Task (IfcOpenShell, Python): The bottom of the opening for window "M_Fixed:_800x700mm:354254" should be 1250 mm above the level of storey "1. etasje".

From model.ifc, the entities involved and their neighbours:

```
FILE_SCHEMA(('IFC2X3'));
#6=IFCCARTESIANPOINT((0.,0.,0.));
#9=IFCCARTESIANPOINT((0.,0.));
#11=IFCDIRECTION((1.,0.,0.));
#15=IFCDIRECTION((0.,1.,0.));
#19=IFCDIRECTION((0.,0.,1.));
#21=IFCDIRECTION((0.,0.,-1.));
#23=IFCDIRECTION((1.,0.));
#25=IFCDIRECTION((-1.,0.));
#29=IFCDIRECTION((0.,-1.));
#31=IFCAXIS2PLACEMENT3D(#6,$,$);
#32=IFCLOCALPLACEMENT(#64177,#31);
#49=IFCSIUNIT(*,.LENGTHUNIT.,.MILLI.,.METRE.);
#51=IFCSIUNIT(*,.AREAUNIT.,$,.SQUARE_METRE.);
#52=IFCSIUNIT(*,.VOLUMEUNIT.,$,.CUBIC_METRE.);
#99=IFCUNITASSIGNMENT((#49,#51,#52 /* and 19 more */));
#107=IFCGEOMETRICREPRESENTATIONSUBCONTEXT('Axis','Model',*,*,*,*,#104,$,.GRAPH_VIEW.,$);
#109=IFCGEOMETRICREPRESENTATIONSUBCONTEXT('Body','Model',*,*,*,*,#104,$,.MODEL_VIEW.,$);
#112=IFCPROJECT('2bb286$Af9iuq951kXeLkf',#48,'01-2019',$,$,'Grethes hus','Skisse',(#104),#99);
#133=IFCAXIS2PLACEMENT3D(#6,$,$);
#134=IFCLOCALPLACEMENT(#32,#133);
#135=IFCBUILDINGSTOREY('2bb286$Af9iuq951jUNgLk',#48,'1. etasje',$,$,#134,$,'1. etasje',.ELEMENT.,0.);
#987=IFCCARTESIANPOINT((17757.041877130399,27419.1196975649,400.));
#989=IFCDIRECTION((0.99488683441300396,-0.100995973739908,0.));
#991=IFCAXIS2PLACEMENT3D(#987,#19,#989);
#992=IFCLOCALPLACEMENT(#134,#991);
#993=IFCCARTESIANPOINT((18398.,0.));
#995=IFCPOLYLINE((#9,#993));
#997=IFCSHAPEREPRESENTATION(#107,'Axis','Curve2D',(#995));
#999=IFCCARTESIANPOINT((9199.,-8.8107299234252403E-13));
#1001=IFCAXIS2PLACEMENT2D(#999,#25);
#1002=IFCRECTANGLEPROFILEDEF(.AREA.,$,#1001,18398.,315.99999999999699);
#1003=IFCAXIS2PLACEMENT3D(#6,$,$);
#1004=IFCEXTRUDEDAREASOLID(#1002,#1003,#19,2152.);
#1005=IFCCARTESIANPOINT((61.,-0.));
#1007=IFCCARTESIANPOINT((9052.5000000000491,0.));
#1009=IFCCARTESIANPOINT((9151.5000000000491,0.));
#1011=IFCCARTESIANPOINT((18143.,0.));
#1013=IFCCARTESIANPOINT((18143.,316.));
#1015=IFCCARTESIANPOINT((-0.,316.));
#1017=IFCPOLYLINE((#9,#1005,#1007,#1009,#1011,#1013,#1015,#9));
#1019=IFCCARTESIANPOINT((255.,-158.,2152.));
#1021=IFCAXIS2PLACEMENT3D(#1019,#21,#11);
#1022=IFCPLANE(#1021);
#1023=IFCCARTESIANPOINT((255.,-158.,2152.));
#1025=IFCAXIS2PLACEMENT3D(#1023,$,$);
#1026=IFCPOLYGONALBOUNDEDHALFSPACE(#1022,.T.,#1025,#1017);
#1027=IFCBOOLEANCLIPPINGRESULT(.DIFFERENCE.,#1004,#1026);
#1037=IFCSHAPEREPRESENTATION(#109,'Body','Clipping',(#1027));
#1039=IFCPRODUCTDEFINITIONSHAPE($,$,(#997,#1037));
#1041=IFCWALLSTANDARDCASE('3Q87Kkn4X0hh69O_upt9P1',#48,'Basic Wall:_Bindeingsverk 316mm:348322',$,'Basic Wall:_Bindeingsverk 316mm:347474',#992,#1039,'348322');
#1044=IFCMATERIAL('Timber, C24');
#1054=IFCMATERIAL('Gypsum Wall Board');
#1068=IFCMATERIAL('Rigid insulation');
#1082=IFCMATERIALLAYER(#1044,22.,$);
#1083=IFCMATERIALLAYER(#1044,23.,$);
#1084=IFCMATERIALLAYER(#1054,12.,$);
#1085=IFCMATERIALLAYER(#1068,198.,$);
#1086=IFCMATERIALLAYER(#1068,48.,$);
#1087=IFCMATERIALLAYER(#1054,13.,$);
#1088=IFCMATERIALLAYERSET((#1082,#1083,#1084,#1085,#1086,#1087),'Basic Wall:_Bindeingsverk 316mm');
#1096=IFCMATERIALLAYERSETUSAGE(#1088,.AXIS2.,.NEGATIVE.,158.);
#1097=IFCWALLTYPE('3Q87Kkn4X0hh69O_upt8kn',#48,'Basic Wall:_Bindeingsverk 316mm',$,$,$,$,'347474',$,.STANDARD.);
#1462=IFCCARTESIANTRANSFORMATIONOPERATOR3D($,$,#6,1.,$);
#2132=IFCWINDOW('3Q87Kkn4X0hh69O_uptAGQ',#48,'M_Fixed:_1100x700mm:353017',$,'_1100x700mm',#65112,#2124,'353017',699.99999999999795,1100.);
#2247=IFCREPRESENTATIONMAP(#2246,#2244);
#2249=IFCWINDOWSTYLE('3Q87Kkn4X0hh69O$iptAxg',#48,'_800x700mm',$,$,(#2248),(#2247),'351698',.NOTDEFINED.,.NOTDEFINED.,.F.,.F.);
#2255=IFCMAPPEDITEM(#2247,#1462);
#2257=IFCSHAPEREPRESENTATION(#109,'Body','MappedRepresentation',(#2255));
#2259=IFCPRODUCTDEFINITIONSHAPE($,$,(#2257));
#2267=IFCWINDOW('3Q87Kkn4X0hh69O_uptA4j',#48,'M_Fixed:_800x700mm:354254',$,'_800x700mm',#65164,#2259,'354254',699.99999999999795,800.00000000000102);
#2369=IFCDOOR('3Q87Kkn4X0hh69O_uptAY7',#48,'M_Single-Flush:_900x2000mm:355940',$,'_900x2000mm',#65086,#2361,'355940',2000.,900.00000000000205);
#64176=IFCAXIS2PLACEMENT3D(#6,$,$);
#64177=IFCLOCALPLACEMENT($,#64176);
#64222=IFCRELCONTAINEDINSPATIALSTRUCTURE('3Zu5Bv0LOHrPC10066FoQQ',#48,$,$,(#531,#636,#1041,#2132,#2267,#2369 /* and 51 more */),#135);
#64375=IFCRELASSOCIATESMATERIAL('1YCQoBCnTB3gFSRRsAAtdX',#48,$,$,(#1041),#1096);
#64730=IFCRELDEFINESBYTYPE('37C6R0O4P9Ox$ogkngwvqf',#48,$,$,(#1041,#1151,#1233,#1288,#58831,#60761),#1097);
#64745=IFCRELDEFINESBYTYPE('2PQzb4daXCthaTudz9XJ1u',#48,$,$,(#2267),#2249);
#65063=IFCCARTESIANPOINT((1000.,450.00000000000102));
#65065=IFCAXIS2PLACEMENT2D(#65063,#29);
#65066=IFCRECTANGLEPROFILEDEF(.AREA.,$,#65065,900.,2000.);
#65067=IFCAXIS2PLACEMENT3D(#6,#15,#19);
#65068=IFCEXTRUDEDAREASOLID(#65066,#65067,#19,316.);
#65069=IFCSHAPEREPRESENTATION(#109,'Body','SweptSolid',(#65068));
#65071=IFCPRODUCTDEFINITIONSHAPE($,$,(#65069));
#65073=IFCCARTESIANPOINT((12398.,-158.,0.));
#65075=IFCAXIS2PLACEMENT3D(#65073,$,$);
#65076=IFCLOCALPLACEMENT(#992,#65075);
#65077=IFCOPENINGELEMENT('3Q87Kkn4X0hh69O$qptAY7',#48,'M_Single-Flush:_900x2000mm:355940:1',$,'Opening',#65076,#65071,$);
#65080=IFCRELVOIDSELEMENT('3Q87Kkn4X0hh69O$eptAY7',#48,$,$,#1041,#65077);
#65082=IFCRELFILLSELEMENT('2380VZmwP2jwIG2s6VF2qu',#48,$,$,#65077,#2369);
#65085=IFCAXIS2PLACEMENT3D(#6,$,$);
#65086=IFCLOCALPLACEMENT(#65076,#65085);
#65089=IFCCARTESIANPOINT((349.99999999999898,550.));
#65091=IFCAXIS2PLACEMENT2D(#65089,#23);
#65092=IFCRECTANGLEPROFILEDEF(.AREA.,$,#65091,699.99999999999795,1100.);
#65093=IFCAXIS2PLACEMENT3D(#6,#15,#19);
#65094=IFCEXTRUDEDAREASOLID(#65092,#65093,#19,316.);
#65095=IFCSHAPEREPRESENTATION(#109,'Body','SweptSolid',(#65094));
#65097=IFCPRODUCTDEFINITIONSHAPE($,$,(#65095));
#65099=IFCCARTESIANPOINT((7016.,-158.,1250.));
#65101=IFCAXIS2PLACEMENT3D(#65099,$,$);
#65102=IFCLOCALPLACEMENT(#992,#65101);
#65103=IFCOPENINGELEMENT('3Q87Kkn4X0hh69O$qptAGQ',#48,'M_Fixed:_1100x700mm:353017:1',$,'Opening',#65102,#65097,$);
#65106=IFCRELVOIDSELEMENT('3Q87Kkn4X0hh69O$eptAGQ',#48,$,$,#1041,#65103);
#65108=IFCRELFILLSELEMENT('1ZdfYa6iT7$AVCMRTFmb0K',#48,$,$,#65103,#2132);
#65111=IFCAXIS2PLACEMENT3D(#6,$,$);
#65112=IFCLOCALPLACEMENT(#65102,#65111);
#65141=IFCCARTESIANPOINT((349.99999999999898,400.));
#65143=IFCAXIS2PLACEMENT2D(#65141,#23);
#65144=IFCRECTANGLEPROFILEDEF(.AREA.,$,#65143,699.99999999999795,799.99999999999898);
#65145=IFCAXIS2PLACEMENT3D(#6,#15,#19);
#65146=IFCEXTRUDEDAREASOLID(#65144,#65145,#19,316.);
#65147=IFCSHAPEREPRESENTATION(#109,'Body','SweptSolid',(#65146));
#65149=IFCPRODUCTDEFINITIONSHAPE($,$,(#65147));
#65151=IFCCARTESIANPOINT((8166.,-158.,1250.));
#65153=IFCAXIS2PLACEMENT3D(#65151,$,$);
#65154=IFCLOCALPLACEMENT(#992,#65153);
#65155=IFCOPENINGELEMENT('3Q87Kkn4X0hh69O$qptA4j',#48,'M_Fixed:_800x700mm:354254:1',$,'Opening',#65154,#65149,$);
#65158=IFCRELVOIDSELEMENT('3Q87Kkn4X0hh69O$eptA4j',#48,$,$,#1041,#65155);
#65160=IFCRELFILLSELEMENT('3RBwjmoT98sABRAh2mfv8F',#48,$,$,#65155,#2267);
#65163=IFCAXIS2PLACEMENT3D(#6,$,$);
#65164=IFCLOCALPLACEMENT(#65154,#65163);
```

```python
import numpy as np
import ifcopenshell
import ifcopenshell.api.geometry
import ifcopenshell.geom
import ifcopenshell.util.element
import ifcopenshell.util.placement
import ifcopenshell.util.shape
import ifcopenshell.util.unit

model = ifcopenshell.open("model.ifc")
unit_scale = ifcopenshell.util.unit.calculate_unit_scale(model)

window = model.by_id(2267)
opening = window.FillsVoids[0].RelatingOpeningElement
storey = ifcopenshell.util.element.get_container(window, ifc_class="IfcBuildingStorey")
level = ifcopenshell.util.placement.get_local_placement(storey.ObjectPlacement)[2, 3]

# The opening's origin need not be at the sill, so measure its lowest point.
shape = ifcopenshell.geom.create_shape(ifcopenshell.geom.settings(), opening)
bottom = ifcopenshell.util.shape.get_shape_bottom_elevation(shape, shape.geometry) / unit_scale
dz = level + 1250.0 - bottom

shift = np.array([0.0, 0.0, dz])
# The window is placed relative to its opening, so it follows when the opening moves.
matrix = ifcopenshell.util.placement.get_local_placement(opening.ObjectPlacement)
matrix[:3, 3] += shift
ifcopenshell.api.geometry.edit_object_placement(
    model, product=opening, matrix=matrix, is_si=False, should_transform_children=True
)

print(f"moved by {dz * unit_scale:+.3f} m")

model.write("model_edited.ifc")
```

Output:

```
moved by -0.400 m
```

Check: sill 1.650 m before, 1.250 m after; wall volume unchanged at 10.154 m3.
